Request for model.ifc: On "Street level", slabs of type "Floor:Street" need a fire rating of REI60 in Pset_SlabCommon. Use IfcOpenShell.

First a look at what the model holds.

```python
import ifcopenshell
import ifcopenshell.util.element

model = ifcopenshell.open("model.ifc")
print(model.schema)
storey = next(s for s in model.by_type("IfcBuildingStorey") if s.Name == "Street level")
slabs = [e for e in ifcopenshell.util.element.get_decomposition(storey) if e.is_a("IfcSlab")]
seen = {}
for e in slabs:
    element_type = ifcopenshell.util.element.get_type(e)
    key = (element_type.Name if element_type != e and element_type else None, ifcopenshell.util.element.get_pset(e, "Pset_SlabCommon", "FireRating"))
    seen[key] = seen.get(key, 0) + 1
for (name, value), count in sorted(seen.items(), key=str):
    print(count, "x", name, "|", value)
```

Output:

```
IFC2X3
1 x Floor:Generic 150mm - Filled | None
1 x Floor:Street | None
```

```python
import ifcopenshell
import ifcopenshell.api.pset
import ifcopenshell.util.element

model = ifcopenshell.open("model.ifc")

storey = next(s for s in model.by_type("IfcBuildingStorey") if s.Name == "Street level")
slabs = [e for e in ifcopenshell.util.element.get_decomposition(storey) if e.is_a("IfcSlab")]

count = 0
for e in slabs:
    element_type = ifcopenshell.util.element.get_type(e)
    if element_type in (None, e) or element_type.Name != "Floor:Street":
        continue
    # add_pset returns the element's existing set when there is one.
    pset = ifcopenshell.api.pset.add_pset(model, product=e, name="Pset_SlabCommon")
    ifcopenshell.api.pset.edit_pset(model, pset=pset, properties={"FireRating": "REI60"})
    count += 1

print(count, "slabs updated")

model.write("model_rev.ifc")
```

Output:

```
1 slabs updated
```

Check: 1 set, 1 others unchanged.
